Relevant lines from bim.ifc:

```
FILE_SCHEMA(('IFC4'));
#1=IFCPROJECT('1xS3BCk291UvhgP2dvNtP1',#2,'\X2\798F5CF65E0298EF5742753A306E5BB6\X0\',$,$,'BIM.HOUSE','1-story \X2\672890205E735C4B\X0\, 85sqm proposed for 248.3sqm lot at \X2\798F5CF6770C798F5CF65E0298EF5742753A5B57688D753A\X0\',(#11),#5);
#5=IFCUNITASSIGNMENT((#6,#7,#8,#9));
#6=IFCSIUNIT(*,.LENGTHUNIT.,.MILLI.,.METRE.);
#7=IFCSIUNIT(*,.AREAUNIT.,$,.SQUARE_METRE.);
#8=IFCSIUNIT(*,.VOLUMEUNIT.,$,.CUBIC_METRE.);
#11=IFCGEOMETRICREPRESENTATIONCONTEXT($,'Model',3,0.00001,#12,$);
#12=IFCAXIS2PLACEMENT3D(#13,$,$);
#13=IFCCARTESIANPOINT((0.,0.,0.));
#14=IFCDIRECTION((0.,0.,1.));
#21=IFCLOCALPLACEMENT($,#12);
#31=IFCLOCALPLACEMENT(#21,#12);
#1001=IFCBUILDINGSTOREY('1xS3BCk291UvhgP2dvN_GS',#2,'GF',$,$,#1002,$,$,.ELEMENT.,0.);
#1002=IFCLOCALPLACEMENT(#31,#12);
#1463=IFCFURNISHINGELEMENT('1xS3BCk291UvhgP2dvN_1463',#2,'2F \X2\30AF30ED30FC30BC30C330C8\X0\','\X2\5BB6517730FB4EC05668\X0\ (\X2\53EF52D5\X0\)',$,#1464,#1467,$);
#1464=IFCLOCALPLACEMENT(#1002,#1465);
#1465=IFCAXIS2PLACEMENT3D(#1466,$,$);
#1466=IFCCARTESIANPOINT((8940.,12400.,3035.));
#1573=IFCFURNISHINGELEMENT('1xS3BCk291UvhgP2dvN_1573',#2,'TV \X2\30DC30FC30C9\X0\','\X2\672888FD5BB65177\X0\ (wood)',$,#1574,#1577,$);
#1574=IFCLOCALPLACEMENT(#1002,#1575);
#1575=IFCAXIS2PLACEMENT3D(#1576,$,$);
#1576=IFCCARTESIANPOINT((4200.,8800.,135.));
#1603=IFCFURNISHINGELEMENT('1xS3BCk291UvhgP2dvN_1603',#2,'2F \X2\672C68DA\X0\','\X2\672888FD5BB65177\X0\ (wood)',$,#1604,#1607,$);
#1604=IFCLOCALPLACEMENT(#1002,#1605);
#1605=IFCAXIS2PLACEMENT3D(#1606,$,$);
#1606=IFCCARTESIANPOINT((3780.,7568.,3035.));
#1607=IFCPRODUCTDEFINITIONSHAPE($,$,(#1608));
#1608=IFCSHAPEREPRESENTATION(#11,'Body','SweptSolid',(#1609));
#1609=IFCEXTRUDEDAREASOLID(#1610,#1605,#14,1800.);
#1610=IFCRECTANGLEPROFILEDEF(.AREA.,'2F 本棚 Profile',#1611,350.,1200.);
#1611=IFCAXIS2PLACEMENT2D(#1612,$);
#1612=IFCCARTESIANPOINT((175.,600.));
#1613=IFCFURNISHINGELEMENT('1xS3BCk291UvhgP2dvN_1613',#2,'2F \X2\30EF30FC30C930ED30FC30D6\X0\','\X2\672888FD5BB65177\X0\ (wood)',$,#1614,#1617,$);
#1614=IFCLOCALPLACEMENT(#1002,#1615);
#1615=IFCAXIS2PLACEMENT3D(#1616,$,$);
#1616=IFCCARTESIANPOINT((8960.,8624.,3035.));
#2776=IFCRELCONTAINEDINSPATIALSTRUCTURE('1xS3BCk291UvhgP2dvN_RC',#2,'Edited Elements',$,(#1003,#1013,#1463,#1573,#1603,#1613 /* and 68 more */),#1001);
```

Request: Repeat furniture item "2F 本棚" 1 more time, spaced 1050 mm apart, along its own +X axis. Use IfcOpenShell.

```python
import ifcopenshell
import ifcopenshell.api.geometry
import ifcopenshell.api.root
import ifcopenshell.util.element
import ifcopenshell.util.placement

model = ifcopenshell.open("bim.ifc")


def reuse_history(source, copy):
    """copy_class also copies each property set's owner history, people and application; keep the originals."""
    for rel in copy.IsDefinedBy:
        if rel.is_a("IfcRelDefinesByProperties") and (history := rel.RelatingPropertyDefinition.OwnerHistory):
            rel.RelatingPropertyDefinition.OwnerHistory = source.OwnerHistory
            ifcopenshell.util.element.remove_deep2(model, history)


source = model.by_guid("1xS3BCk291UvhgP2dvN_1603")
base = ifcopenshell.util.placement.get_local_placement(source.ObjectPlacement)
step = base[:3, 0] * 1050.0

for i in range(1, 2):
    copy = ifcopenshell.api.root.copy_class(model, product=source)
    copy.Representation = ifcopenshell.util.element.copy_deep(
        model, source.Representation, exclude=["IfcGeometricRepresentationContext", "IfcRepresentationMap"]
    )
    reuse_history(source, copy)
    matrix = base.copy()
    matrix[:3, 3] += i * step
    print("added at", matrix[:3, 3].round(3) + 0.0)
    ifcopenshell.api.geometry.edit_object_placement(model, product=copy, matrix=matrix, is_si=False)

model.write("bim_updated.ifc")
```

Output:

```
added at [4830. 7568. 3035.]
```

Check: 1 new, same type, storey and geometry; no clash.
